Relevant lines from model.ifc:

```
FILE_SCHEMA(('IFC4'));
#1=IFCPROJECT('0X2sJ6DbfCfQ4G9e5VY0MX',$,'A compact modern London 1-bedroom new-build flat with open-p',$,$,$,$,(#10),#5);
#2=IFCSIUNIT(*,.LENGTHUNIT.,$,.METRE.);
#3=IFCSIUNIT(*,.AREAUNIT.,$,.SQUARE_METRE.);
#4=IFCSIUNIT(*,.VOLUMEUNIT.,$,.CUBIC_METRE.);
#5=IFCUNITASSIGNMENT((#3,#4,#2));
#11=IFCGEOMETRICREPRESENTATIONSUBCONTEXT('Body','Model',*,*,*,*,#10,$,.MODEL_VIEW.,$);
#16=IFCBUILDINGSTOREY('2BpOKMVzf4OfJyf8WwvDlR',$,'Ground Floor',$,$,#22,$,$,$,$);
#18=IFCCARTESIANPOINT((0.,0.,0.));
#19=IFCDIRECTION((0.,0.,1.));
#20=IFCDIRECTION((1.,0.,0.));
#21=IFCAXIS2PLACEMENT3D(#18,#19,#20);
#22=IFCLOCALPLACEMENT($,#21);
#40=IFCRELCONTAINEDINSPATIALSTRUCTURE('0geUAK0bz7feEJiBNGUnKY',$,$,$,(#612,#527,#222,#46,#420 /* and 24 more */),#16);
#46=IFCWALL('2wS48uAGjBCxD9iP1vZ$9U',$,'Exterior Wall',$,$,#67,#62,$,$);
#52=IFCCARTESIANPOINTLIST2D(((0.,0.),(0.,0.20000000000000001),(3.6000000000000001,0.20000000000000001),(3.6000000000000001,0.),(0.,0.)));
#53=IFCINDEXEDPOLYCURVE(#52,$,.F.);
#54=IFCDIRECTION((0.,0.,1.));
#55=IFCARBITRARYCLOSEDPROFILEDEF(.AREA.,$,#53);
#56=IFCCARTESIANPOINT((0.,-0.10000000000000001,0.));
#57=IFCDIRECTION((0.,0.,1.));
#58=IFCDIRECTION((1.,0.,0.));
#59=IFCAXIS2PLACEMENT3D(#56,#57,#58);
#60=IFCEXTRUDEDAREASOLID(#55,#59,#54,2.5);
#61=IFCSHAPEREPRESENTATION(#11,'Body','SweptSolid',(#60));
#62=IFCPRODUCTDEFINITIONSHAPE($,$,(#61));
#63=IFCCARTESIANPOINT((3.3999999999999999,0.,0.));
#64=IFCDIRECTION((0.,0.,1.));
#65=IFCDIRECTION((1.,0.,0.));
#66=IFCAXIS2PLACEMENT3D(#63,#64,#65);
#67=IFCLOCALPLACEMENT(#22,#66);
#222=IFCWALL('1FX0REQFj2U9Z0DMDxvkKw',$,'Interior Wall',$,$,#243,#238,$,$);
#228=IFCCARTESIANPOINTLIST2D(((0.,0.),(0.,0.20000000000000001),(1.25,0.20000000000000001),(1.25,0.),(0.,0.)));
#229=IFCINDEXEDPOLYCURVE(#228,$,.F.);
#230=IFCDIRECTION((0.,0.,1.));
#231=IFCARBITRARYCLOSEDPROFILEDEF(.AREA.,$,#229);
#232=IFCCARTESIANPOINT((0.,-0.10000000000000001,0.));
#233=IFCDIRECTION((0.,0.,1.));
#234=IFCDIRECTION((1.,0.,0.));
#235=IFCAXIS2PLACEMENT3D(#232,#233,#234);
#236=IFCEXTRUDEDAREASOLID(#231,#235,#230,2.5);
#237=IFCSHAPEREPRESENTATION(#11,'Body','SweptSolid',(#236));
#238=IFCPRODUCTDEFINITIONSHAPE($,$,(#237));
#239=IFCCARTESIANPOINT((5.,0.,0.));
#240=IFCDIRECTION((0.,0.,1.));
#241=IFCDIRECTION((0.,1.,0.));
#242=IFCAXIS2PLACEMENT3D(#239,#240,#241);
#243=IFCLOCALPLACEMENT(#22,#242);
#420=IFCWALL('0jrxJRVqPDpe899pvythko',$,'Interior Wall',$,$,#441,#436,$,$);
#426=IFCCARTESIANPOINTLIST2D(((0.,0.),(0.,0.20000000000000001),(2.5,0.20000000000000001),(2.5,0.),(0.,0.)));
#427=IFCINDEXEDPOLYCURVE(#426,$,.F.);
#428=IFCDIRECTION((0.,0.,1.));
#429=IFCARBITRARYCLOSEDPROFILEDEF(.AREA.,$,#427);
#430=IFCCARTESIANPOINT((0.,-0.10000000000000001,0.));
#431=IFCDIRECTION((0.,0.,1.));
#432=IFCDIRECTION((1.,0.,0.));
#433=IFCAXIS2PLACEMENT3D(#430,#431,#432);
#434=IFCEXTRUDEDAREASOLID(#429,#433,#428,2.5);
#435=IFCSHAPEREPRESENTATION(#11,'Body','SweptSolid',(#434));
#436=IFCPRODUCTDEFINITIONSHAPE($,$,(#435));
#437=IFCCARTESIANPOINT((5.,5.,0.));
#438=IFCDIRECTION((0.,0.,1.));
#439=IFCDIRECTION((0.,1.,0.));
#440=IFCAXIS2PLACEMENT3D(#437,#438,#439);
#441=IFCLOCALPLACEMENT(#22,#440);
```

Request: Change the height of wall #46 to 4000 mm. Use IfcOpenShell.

```python
import ifcopenshell
import ifcopenshell.geom
import ifcopenshell.util.representation
import ifcopenshell.util.shape

model = ifcopenshell.open("model.ifc")
settings = ifcopenshell.geom.settings()


def volume(element):
    """Net volume in cubic metres, openings subtracted."""
    shape = ifcopenshell.geom.create_shape(settings, element)
    return ifcopenshell.util.shape.get_volume(shape.geometry)


wall = model.by_id(46)
before = volume(wall)

body = ifcopenshell.util.representation.get_representation(wall, "Model", "Body")
solid = body.Items[0]
old_height = solid.Depth
solid.Depth = 4.0
after = volume(wall)

print(f"height {old_height:g} -> {solid.Depth:g}, volume {before:.3f} -> {after:.3f} m3")

model.write("model_updated.ifc")
```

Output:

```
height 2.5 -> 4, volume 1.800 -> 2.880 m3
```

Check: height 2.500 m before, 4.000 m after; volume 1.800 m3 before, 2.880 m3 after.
